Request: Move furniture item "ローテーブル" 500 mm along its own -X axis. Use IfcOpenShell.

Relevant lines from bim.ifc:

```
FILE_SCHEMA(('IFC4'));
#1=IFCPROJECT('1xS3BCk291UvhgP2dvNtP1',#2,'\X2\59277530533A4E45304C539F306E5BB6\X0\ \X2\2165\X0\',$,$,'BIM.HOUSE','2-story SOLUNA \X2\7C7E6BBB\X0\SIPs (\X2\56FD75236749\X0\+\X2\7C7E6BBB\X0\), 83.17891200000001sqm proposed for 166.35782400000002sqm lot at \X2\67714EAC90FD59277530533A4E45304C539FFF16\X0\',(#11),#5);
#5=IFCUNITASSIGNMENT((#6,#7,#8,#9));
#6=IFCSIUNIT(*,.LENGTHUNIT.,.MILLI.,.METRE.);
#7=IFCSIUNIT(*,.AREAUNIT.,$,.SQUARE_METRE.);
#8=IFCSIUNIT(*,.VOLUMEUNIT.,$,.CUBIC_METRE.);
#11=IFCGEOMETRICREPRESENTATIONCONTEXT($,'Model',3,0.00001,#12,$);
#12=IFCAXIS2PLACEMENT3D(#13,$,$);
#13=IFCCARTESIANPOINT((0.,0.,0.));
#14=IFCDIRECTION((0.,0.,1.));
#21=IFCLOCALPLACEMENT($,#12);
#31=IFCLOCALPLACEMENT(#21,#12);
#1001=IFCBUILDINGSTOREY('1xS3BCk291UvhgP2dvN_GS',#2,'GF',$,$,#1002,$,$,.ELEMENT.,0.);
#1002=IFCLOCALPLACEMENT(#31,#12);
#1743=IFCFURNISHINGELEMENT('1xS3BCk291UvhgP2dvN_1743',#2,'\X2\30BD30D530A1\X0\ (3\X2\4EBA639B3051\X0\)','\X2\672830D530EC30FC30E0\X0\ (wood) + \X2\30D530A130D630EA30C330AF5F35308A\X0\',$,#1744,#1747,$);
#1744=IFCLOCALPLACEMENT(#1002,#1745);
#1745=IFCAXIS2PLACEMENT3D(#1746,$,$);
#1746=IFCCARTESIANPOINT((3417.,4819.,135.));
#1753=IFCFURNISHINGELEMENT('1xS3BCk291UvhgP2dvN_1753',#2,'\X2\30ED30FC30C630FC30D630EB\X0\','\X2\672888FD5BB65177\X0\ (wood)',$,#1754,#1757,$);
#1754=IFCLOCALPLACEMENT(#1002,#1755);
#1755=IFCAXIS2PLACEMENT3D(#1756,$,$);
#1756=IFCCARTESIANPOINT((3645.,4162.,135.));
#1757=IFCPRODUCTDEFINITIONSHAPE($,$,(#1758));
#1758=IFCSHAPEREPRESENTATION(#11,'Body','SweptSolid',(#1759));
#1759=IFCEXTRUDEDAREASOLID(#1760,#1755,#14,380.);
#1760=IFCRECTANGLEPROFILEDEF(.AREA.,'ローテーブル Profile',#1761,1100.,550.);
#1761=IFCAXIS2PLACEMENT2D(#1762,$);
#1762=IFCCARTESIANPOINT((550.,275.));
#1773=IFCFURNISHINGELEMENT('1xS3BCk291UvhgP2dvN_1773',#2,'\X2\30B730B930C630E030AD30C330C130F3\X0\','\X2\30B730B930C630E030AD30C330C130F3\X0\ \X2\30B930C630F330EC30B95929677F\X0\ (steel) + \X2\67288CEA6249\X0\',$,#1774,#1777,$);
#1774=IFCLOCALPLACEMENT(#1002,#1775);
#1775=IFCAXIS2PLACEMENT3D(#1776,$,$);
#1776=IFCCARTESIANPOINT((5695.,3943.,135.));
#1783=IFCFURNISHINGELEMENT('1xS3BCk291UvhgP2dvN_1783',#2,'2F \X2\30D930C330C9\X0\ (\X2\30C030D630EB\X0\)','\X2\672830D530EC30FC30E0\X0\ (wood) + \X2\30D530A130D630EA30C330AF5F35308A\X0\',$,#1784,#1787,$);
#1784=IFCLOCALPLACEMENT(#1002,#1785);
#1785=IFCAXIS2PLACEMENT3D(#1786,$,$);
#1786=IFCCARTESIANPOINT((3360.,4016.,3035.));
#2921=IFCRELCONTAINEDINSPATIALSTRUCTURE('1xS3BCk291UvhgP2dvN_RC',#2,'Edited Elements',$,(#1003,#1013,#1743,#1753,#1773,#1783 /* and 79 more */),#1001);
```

```python
import ifcopenshell
import ifcopenshell.api.geometry
import ifcopenshell.util.placement
import ifcopenshell.util.unit

model = ifcopenshell.open("bim.ifc")
unit_scale = ifcopenshell.util.unit.calculate_unit_scale(model)

item = model.by_guid("1xS3BCk291UvhgP2dvN_1753")
matrix = ifcopenshell.util.placement.get_local_placement(item.ObjectPlacement)
matrix[:3, 3] -= matrix[:3, 0] * 0.5 / unit_scale
ifcopenshell.api.geometry.edit_object_placement(model, product=item, matrix=matrix, is_si=False)

print(ifcopenshell.util.placement.get_local_placement(item.ObjectPlacement).round(3) + 0.0)

model.write("bim-out.ifc")
```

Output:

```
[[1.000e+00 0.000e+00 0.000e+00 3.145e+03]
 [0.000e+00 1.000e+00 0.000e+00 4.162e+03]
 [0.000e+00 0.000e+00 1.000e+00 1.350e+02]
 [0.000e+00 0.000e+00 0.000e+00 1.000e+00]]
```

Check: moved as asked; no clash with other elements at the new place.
